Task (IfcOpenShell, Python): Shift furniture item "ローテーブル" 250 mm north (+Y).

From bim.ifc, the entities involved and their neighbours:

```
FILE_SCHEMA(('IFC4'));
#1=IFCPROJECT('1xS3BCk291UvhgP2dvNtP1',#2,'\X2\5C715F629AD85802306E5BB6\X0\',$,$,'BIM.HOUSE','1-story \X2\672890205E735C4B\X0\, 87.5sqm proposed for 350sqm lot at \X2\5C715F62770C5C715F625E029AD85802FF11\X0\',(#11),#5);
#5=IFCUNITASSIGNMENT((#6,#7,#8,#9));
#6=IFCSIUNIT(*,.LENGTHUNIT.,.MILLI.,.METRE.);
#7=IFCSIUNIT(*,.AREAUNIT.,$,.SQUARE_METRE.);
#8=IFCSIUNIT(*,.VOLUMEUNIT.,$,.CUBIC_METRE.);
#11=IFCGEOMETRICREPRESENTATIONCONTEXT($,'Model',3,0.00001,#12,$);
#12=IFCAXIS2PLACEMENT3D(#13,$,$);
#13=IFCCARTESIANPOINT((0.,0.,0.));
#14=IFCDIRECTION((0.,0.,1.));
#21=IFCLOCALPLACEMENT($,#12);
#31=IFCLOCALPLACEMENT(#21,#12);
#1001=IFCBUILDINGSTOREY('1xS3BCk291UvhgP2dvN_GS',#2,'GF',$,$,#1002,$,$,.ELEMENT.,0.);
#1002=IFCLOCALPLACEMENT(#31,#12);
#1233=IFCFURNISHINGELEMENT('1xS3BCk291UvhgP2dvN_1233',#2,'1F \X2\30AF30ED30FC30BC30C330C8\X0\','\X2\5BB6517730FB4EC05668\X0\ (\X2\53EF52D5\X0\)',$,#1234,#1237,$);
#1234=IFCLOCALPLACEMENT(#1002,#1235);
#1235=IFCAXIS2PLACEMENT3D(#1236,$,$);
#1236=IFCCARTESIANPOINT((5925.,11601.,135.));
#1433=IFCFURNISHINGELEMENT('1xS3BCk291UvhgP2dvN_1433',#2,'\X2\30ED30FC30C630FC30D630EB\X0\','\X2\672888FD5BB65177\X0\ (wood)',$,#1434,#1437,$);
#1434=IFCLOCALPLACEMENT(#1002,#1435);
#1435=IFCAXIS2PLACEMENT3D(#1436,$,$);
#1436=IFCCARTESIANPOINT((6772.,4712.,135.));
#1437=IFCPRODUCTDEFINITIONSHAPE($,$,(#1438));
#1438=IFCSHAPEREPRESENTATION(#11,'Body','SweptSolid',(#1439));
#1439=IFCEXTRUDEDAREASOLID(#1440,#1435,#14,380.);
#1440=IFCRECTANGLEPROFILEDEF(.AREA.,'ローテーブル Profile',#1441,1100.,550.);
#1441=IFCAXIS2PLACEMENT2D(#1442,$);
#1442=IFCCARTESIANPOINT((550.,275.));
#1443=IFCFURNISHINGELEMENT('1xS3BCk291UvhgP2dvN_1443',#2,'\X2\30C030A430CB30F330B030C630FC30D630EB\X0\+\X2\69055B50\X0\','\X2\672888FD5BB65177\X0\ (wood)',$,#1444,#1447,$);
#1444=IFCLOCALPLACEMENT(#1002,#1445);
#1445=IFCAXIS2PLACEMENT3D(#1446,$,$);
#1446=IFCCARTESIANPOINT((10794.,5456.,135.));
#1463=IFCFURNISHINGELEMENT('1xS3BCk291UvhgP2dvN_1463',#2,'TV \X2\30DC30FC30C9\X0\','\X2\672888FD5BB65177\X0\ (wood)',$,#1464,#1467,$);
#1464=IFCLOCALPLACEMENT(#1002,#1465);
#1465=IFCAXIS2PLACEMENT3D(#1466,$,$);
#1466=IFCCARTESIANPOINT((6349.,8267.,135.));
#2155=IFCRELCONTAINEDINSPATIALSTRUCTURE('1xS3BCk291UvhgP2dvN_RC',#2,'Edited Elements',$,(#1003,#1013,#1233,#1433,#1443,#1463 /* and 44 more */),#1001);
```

```python
import ifcopenshell
import ifcopenshell.api.geometry
import ifcopenshell.util.placement
import ifcopenshell.util.unit

model = ifcopenshell.open("bim.ifc")
unit_scale = ifcopenshell.util.unit.calculate_unit_scale(model)

item = model.by_guid("1xS3BCk291UvhgP2dvN_1433")
matrix = ifcopenshell.util.placement.get_local_placement(item.ObjectPlacement)
matrix[1, 3] += 0.25 / unit_scale
ifcopenshell.api.geometry.edit_object_placement(model, product=item, matrix=matrix, is_si=False)

print(ifcopenshell.util.placement.get_local_placement(item.ObjectPlacement).round(3) + 0.0)

model.write("bim_edited.ifc")
```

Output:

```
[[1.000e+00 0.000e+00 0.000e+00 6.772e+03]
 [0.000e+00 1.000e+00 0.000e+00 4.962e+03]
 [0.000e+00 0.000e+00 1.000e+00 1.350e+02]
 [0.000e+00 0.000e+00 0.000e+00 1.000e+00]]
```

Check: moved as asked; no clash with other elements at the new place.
